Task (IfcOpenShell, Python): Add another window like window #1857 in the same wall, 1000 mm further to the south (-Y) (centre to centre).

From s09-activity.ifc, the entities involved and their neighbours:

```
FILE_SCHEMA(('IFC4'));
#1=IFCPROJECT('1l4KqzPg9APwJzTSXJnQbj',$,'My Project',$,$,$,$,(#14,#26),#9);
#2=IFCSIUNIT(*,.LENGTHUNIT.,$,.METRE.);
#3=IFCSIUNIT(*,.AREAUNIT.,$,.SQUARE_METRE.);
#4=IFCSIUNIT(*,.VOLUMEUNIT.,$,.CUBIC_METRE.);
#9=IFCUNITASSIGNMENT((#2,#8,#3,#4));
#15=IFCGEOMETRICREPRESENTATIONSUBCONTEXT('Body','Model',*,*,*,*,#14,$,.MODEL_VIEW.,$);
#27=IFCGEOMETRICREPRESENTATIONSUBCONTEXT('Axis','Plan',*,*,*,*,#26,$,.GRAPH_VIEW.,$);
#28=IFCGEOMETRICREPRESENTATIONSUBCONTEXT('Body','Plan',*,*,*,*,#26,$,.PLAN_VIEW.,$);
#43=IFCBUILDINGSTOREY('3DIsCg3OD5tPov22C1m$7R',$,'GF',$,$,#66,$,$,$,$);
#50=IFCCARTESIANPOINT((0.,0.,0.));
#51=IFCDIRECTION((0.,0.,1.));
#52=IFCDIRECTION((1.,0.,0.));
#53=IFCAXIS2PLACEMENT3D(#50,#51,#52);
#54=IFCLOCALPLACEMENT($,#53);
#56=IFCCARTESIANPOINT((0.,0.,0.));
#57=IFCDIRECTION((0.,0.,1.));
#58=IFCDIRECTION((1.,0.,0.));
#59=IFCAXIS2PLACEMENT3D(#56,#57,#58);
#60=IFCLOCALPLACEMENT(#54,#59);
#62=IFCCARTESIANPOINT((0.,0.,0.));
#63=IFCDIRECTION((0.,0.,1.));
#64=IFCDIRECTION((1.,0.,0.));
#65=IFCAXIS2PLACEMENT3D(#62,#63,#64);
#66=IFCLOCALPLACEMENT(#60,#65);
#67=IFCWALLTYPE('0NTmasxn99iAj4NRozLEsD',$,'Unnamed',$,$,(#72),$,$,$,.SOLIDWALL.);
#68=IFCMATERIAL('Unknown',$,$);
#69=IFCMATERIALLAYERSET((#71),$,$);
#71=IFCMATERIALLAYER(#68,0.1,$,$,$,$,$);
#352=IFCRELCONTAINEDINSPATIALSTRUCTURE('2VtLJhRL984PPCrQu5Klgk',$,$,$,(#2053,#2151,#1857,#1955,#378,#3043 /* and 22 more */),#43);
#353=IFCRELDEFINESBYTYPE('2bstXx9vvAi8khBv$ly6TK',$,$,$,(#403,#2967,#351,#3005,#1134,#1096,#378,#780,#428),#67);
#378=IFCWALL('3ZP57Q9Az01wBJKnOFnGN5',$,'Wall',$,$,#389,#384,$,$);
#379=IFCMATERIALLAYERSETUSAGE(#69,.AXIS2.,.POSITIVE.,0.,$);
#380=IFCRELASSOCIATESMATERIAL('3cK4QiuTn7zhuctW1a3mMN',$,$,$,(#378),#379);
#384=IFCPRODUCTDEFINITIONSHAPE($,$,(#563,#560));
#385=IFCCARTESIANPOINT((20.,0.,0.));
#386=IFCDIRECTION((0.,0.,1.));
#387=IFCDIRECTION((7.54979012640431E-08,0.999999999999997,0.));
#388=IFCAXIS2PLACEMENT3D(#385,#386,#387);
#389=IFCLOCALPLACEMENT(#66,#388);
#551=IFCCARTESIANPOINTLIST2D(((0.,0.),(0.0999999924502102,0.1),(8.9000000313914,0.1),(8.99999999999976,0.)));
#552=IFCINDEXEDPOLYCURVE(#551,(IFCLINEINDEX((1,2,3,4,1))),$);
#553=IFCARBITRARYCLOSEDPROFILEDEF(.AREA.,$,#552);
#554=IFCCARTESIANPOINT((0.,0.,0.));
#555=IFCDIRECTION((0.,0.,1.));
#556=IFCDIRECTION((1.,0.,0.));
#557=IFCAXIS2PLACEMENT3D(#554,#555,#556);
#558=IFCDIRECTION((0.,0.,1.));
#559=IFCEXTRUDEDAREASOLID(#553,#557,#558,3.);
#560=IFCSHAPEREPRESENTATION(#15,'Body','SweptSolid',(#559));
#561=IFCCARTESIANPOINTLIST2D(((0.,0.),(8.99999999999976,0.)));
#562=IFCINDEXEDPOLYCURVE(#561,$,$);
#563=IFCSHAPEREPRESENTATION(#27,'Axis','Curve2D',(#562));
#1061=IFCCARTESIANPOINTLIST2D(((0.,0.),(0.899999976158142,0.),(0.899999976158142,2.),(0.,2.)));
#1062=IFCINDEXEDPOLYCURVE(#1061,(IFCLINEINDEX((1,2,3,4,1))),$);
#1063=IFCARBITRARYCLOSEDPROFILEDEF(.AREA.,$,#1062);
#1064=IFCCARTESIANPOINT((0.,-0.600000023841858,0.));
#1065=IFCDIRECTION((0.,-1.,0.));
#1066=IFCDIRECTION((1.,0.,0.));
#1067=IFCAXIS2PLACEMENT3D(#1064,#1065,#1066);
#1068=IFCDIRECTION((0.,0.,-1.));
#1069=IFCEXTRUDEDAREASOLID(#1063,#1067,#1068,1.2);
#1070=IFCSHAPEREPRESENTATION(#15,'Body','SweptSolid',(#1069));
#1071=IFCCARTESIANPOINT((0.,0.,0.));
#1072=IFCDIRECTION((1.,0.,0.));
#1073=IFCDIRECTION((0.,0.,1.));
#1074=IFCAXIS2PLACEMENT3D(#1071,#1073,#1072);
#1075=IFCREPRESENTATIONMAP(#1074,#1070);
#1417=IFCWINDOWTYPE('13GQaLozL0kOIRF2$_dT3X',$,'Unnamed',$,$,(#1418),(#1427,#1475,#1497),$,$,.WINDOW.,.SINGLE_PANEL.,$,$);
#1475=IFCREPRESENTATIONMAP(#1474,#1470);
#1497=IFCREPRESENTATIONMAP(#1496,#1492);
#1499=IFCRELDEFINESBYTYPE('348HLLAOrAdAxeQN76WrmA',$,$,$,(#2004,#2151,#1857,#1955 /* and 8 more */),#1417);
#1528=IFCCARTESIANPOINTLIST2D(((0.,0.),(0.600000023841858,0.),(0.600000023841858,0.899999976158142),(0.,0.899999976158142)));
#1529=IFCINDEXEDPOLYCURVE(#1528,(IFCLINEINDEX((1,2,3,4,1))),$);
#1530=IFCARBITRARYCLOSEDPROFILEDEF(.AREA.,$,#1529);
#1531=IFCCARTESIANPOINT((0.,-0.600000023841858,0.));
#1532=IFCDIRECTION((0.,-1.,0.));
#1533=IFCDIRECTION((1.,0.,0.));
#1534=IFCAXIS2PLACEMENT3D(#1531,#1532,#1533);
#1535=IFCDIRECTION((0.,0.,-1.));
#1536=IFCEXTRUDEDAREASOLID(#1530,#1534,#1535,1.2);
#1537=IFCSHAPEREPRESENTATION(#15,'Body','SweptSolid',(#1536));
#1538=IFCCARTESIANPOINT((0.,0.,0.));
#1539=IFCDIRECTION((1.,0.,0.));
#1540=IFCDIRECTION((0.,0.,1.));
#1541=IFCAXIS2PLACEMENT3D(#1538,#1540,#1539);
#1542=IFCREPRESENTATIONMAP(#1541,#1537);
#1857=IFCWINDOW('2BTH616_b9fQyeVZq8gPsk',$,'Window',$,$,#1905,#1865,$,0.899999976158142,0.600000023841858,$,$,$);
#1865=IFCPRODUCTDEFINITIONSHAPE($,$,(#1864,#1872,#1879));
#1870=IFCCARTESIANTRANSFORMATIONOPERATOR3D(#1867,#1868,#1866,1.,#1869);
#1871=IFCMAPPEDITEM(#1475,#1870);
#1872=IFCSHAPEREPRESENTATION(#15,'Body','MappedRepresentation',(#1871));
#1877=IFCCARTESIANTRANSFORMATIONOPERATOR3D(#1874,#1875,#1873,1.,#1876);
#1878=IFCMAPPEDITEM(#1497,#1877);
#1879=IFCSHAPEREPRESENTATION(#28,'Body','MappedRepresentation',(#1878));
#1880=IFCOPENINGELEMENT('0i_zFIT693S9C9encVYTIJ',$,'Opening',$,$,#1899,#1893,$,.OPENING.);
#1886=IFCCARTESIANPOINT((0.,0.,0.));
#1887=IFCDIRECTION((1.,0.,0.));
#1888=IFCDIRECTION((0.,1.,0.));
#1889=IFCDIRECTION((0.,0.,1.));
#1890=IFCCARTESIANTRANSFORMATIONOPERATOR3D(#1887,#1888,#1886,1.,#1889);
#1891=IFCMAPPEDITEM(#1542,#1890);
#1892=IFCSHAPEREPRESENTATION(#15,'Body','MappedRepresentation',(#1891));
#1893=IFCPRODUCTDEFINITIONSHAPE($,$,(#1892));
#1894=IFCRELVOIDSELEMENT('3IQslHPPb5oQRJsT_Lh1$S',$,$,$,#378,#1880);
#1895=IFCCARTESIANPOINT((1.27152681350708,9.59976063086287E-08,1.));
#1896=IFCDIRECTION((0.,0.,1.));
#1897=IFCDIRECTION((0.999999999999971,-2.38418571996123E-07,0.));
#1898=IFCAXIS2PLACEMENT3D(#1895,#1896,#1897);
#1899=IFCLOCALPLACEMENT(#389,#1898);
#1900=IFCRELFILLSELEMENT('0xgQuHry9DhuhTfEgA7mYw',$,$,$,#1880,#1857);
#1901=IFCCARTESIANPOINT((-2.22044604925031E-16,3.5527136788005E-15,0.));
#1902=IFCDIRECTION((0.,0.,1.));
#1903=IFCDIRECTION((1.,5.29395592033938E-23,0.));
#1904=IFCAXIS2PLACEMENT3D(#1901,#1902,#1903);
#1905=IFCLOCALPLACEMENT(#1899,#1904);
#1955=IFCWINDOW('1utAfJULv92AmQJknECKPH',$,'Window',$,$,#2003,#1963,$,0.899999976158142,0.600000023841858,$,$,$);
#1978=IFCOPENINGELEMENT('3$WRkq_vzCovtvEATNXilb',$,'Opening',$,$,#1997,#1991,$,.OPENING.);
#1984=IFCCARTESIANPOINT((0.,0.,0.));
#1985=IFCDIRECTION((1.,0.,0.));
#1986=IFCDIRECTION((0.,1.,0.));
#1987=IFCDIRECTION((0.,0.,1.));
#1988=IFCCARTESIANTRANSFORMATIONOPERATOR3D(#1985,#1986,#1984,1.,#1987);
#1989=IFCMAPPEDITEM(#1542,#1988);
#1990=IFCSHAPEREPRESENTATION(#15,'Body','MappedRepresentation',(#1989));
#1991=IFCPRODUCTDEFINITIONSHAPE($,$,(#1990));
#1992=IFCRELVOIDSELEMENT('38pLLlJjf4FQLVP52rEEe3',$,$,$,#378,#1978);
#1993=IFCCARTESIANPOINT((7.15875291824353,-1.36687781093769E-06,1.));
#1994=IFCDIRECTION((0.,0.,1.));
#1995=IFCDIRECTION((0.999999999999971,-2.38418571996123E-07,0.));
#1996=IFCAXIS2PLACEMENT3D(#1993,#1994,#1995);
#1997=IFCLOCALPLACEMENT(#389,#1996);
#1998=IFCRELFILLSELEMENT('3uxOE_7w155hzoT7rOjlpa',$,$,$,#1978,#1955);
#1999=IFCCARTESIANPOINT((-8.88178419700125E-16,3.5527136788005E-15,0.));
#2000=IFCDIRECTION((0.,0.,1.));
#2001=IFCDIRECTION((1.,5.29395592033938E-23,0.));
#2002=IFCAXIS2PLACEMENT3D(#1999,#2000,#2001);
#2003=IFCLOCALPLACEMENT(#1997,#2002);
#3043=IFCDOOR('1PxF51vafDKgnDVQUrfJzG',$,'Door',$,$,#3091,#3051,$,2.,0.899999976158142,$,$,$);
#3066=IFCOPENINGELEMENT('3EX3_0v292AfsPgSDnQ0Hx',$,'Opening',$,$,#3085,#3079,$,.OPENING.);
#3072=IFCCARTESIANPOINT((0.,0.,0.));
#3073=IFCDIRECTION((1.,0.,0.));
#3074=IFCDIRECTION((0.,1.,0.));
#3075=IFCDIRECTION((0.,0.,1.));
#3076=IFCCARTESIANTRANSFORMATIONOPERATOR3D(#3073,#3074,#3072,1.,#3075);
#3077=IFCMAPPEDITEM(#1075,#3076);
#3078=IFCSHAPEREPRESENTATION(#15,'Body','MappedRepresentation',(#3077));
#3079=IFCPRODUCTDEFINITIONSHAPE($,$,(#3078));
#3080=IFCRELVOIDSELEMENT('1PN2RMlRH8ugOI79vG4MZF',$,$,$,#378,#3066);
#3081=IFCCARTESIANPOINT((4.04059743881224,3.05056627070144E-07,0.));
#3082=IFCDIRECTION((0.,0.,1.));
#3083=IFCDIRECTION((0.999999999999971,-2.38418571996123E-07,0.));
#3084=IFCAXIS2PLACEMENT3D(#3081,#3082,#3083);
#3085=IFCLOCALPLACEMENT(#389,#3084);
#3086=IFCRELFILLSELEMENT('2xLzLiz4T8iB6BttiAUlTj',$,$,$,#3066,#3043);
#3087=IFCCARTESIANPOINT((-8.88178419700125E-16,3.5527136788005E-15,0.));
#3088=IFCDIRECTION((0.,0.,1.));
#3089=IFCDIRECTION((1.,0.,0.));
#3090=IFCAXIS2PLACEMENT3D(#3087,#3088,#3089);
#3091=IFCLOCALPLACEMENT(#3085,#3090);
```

```python
import ifcopenshell
import ifcopenshell.api.feature
import ifcopenshell.api.geometry
import ifcopenshell.api.root
import ifcopenshell.geom
import ifcopenshell.util.element
import ifcopenshell.util.placement
import ifcopenshell.util.shape

model = ifcopenshell.open("s09-activity.ifc")
settings = ifcopenshell.geom.settings()


def volume(element):
    """Net volume in cubic metres, openings subtracted."""
    shape = ifcopenshell.geom.create_shape(settings, element)
    return ifcopenshell.util.shape.get_volume(shape.geometry)


window = model.by_id(1857)
opening = window.FillsVoids[0].RelatingOpeningElement
wall = opening.VoidsElements[0].RelatingBuildingElement
before = volume(wall)
shift = ifcopenshell.util.placement.get_local_placement(wall.ObjectPlacement)[:3, 0] * -1.0

# copy_class copies the void relationship, type, container and properties, but no geometry.
new_opening = ifcopenshell.api.root.copy_class(model, product=opening)
new_opening.Representation = ifcopenshell.util.element.copy_deep(
    model, opening.Representation, exclude=["IfcGeometricRepresentationContext", "IfcRepresentationMap"]
)
new_window = ifcopenshell.api.root.copy_class(model, product=window)
new_window.Representation = ifcopenshell.util.element.copy_deep(
    model, window.Representation, exclude=["IfcGeometricRepresentationContext", "IfcRepresentationMap"]
)
ifcopenshell.api.feature.add_filling(model, opening=new_opening, element=new_window)

for old, new in ((opening, new_opening), (window, new_window)):
    matrix = ifcopenshell.util.placement.get_local_placement(old.ObjectPlacement)
    matrix[:3, 3] += shift
    ifcopenshell.api.geometry.edit_object_placement(model, product=new, matrix=matrix, is_si=False)

after = volume(wall)

print(f"wall volume {before:.3f} -> {after:.3f} m3")

model.write("s09-activity_v2.ifc")
```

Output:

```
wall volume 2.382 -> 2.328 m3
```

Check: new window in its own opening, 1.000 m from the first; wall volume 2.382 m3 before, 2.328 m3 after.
